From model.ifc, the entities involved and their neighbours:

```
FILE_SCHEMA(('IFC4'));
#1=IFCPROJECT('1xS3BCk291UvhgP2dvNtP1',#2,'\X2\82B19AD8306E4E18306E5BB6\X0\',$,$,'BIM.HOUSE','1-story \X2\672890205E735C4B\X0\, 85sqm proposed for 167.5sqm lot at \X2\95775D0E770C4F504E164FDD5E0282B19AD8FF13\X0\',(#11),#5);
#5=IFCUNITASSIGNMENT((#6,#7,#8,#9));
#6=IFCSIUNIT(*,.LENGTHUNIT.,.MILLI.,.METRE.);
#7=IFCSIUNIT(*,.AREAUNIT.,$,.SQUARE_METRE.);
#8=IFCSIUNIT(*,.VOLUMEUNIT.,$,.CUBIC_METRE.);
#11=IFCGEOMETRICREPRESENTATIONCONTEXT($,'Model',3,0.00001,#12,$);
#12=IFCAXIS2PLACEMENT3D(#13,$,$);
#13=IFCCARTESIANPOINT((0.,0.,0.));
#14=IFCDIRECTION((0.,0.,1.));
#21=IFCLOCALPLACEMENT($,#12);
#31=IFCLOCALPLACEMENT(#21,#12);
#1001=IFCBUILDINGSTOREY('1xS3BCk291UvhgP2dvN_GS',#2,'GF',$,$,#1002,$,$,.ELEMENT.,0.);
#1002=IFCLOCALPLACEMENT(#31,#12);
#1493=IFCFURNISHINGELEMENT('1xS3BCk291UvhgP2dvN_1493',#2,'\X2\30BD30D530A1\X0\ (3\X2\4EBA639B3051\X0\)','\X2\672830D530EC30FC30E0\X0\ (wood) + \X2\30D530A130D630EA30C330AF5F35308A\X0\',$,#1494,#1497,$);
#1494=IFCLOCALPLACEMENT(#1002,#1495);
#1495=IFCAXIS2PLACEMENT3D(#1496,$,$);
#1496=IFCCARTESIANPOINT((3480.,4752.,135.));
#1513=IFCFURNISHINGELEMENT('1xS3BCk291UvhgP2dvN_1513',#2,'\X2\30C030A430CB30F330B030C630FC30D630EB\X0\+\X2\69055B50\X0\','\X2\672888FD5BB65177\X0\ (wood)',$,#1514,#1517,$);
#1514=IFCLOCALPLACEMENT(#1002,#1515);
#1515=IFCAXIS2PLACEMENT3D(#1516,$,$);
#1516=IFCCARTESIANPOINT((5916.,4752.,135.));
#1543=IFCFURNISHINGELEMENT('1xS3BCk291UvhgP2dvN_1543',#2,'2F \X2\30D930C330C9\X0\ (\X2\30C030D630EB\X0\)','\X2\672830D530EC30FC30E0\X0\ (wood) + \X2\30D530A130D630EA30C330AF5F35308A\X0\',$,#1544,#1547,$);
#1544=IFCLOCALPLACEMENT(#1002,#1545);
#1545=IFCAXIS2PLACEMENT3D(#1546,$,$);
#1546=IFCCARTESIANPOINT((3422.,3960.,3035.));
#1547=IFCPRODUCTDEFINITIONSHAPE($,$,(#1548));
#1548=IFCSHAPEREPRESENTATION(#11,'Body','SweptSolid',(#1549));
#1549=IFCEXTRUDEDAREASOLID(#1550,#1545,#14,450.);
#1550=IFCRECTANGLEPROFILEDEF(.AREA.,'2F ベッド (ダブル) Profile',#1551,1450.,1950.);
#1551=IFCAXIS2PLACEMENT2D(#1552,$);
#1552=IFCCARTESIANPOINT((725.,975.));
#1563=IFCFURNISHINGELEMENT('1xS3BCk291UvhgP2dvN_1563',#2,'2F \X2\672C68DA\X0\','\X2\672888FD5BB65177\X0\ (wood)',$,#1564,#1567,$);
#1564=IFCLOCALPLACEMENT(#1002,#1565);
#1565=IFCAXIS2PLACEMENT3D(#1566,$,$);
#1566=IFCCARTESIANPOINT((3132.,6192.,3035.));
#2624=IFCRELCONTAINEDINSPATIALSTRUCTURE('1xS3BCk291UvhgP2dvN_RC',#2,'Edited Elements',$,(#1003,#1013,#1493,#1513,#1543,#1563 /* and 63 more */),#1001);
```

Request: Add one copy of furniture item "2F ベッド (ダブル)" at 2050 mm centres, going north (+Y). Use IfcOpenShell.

```python
import numpy as np
import ifcopenshell
import ifcopenshell.api.geometry
import ifcopenshell.api.root
import ifcopenshell.util.element
import ifcopenshell.util.placement
import ifcopenshell.util.unit

model = ifcopenshell.open("model.ifc")
unit_scale = ifcopenshell.util.unit.calculate_unit_scale(model)


def reuse_history(source, copy):
    """copy_class also copies each property set's owner history, people and application; keep the originals."""
    for rel in copy.IsDefinedBy:
        if rel.is_a("IfcRelDefinesByProperties") and (history := rel.RelatingPropertyDefinition.OwnerHistory):
            rel.RelatingPropertyDefinition.OwnerHistory = source.OwnerHistory
            ifcopenshell.util.element.remove_deep2(model, history)


source = model.by_id(1543)
base = ifcopenshell.util.placement.get_local_placement(source.ObjectPlacement)
step = np.array([0.0, 1.0, 0.0]) * 2.05 / unit_scale

for i in range(1, 2):
    copy = ifcopenshell.api.root.copy_class(model, product=source)
    copy.Representation = ifcopenshell.util.element.copy_deep(
        model, source.Representation, exclude=["IfcGeometricRepresentationContext", "IfcRepresentationMap"]
    )
    reuse_history(source, copy)
    matrix = base.copy()
    matrix[:3, 3] += i * step
    print("added at", matrix[:3, 3].round(3) + 0.0)
    ifcopenshell.api.geometry.edit_object_placement(model, product=copy, matrix=matrix, is_si=False)

model.write("model_updated.ifc")
```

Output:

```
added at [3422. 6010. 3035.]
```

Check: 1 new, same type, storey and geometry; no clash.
